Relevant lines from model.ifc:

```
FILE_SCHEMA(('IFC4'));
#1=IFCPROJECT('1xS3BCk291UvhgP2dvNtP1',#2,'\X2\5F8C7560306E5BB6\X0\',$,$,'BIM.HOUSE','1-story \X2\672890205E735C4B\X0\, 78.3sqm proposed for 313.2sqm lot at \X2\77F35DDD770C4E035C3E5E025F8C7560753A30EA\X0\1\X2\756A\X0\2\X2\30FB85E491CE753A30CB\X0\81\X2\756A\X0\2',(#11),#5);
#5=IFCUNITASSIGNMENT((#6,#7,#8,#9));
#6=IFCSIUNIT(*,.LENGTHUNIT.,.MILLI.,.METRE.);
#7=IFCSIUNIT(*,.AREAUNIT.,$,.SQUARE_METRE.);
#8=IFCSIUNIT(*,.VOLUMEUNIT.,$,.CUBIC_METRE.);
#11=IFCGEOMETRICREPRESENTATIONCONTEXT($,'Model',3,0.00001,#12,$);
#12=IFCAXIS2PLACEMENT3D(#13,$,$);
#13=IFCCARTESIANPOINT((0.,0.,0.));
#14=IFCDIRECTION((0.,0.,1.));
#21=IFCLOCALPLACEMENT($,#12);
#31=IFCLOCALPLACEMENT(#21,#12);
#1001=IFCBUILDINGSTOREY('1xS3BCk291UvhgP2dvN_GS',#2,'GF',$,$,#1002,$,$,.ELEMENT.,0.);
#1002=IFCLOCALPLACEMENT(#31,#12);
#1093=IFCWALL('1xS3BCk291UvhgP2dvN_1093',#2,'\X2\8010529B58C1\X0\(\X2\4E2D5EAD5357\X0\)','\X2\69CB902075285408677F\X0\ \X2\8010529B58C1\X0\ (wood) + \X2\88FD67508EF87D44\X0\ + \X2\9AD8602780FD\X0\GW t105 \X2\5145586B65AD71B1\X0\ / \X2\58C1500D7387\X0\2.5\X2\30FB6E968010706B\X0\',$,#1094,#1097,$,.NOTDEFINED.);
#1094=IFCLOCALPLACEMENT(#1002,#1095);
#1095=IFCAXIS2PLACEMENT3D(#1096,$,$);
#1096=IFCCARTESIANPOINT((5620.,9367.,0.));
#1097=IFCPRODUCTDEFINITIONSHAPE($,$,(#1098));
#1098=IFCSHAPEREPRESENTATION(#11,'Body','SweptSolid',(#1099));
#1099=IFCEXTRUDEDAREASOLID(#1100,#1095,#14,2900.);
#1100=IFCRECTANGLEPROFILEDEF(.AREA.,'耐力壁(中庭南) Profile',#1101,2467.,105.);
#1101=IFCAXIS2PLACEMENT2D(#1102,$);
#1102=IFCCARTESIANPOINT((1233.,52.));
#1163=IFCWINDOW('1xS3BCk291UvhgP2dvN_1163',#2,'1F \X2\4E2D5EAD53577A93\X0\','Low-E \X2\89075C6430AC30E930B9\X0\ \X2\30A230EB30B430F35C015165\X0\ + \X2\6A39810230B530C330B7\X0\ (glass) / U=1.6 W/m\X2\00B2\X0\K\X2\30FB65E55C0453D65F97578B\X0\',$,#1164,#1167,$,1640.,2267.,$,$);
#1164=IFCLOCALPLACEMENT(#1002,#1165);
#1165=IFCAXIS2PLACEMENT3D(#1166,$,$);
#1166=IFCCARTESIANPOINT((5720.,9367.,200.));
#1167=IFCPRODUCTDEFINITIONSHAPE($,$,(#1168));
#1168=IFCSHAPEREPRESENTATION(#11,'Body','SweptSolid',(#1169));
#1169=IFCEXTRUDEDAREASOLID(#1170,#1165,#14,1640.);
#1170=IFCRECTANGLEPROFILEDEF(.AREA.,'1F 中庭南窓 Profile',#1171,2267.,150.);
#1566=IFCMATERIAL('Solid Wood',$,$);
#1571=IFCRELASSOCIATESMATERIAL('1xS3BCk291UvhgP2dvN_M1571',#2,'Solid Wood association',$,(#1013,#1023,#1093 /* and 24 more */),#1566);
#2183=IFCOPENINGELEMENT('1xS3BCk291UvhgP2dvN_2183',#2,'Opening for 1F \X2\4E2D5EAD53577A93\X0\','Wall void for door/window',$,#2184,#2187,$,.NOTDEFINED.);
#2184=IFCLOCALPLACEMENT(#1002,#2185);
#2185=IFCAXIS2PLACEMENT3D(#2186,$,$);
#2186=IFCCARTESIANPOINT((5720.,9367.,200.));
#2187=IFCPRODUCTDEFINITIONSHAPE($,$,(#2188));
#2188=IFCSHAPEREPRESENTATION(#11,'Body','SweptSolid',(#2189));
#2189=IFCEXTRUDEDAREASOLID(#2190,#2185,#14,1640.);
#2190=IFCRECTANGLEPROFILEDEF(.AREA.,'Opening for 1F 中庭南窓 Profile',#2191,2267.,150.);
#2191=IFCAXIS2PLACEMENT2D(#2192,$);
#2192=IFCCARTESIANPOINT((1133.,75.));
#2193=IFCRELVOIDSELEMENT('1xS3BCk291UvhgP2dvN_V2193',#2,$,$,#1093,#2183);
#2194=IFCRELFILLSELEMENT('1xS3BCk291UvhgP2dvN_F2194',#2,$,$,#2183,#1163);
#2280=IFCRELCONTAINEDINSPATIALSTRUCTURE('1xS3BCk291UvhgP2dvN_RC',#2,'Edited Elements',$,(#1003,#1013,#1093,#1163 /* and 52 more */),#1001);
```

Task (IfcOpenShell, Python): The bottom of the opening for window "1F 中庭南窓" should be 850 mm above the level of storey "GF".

```python
import numpy as np
import ifcopenshell
import ifcopenshell.api.geometry
import ifcopenshell.geom
import ifcopenshell.util.element
import ifcopenshell.util.placement
import ifcopenshell.util.shape
import ifcopenshell.util.unit

model = ifcopenshell.open("model.ifc")
unit_scale = ifcopenshell.util.unit.calculate_unit_scale(model)

window = model.by_guid("1xS3BCk291UvhgP2dvN_1163")
opening = window.FillsVoids[0].RelatingOpeningElement
storey = ifcopenshell.util.element.get_container(window, ifc_class="IfcBuildingStorey")
level = ifcopenshell.util.placement.get_local_placement(storey.ObjectPlacement)[2, 3]

# The opening's origin need not be at the sill, so measure its lowest point.
shape = ifcopenshell.geom.create_shape(ifcopenshell.geom.settings(), opening)
bottom = ifcopenshell.util.shape.get_shape_bottom_elevation(shape, shape.geometry) / unit_scale
dz = level + 0.85 / unit_scale - bottom

shift = np.array([0.0, 0.0, dz])
# The window is not placed relative to its opening, so move both.
for product in (opening, window):
    matrix = ifcopenshell.util.placement.get_local_placement(product.ObjectPlacement)
    matrix[:3, 3] += shift
    ifcopenshell.api.geometry.edit_object_placement(model, product=product, matrix=matrix, is_si=False)

print(f"moved by {dz * unit_scale:+.3f} m")

model.write("model_v2.ifc")
```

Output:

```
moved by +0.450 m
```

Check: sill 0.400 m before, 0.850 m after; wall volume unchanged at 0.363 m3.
